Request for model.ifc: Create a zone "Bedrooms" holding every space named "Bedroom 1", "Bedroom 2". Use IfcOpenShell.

First a look at what the model holds.

```python
import ifcopenshell

model = ifcopenshell.open("model.ifc")
print(model.schema)
seen = {}
for space in model.by_type("IfcSpace"):
    seen[space.LongName] = seen.get(space.LongName, 0) + 1
for name, count in sorted(seen.items(), key=str):
    print(count, "x", name)
print("zones:", [z.Name for z in model.by_type("IfcZone")][:20])
```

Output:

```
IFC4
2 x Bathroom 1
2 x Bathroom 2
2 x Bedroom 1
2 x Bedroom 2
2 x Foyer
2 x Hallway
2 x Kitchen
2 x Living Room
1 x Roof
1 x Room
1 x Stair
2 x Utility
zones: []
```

```python
import ifcopenshell
import ifcopenshell.api.group
import ifcopenshell.api.root

model = ifcopenshell.open("model.ifc")

names = {"Bedroom 1", "Bedroom 2"}
spaces = [s for s in model.by_type("IfcSpace") if s.LongName in names]

zone = ifcopenshell.api.root.create_entity(model, ifc_class="IfcZone", name="Bedrooms")
ifcopenshell.api.group.assign_group(model, products=spaces, group=zone)
print(len(spaces), "spaces in", zone.Name)

model.write("model_rev.ifc")
```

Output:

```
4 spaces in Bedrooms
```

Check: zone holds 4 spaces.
